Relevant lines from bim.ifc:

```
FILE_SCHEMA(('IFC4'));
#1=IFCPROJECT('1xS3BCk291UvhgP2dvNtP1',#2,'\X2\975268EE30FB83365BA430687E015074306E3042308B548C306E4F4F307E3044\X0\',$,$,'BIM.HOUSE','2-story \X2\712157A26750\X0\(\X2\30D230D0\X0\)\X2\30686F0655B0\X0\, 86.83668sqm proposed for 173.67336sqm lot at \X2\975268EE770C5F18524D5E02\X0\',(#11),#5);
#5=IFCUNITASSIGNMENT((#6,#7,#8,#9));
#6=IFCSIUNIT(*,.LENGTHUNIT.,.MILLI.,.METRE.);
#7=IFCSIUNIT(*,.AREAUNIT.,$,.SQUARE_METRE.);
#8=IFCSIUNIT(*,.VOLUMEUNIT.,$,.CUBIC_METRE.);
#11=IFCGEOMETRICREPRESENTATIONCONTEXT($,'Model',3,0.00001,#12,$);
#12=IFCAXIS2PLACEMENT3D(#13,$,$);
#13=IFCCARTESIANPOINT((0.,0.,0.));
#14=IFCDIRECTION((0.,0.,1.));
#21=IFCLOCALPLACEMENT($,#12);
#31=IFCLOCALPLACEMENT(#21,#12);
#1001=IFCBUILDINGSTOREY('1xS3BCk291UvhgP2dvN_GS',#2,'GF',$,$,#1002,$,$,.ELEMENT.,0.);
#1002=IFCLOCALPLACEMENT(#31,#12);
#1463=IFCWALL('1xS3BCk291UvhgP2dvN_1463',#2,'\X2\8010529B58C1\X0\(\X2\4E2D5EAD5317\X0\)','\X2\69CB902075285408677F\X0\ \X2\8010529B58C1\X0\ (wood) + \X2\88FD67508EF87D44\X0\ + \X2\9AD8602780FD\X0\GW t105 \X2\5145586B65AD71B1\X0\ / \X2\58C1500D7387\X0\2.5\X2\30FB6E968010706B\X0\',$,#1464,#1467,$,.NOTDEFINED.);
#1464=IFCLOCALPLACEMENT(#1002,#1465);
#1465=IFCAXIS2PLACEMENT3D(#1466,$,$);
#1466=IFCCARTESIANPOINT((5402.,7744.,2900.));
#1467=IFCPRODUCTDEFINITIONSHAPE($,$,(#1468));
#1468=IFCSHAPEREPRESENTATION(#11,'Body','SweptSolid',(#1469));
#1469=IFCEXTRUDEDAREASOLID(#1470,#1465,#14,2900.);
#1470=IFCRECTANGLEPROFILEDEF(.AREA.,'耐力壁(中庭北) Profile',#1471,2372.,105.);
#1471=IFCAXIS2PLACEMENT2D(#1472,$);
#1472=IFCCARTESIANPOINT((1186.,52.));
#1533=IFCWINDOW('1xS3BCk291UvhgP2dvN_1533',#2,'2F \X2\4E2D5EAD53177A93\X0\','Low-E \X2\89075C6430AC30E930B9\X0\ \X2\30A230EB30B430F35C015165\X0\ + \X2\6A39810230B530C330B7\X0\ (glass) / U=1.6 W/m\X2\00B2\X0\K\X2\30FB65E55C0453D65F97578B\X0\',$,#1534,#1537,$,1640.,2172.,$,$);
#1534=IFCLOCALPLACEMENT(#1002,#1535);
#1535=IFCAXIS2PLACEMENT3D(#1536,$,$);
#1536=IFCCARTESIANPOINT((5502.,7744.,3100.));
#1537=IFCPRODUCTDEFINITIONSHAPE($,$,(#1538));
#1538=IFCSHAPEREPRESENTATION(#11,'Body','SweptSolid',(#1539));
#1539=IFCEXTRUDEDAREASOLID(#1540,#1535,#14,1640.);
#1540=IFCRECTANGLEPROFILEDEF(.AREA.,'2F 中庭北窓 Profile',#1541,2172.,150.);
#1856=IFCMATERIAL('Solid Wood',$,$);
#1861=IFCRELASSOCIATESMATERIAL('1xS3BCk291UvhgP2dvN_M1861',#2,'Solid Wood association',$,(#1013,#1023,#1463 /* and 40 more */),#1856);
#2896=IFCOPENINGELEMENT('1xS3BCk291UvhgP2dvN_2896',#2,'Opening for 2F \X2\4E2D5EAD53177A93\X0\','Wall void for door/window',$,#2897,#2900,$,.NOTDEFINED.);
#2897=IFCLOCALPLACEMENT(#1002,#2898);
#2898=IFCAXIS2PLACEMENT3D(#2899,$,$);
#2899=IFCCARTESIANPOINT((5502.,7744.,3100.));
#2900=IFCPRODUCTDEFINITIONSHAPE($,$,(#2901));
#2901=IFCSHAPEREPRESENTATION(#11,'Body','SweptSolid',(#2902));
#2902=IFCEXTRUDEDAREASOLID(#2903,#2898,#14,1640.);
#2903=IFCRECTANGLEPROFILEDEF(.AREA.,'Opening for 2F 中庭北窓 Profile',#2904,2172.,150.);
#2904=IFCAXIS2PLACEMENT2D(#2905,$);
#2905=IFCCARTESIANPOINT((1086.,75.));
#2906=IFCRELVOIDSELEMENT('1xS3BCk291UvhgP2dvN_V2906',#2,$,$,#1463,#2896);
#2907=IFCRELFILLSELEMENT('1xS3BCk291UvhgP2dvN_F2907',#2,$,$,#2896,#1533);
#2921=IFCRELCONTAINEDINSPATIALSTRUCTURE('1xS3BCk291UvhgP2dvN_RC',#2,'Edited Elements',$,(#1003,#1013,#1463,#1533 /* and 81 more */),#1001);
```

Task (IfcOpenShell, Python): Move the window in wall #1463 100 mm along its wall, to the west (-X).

```python
import ifcopenshell
import ifcopenshell.api.geometry
import ifcopenshell.util.placement
import ifcopenshell.util.unit

model = ifcopenshell.open("bim.ifc")
unit_scale = ifcopenshell.util.unit.calculate_unit_scale(model)

window = model.by_guid("1xS3BCk291UvhgP2dvN_1533")
opening = window.FillsVoids[0].RelatingOpeningElement
wall = opening.VoidsElements[0].RelatingBuildingElement

wall_matrix = ifcopenshell.util.placement.get_local_placement(wall.ObjectPlacement)
shift = wall_matrix[:3, 0] * -0.1 / unit_scale
before = ifcopenshell.util.placement.get_local_placement(window.ObjectPlacement)[:3, 3].copy()

# The window is not placed relative to its opening, so move both.
for product in (opening, window):
    matrix = ifcopenshell.util.placement.get_local_placement(product.ObjectPlacement)
    matrix[:3, 3] += shift
    ifcopenshell.api.geometry.edit_object_placement(model, product=product, matrix=matrix, is_si=False)

after = ifcopenshell.util.placement.get_local_placement(window.ObjectPlacement)[:3, 3]
print("window moved by", (after - before).round(3) + 0.0)

model.write("bim_v2.ifc")
```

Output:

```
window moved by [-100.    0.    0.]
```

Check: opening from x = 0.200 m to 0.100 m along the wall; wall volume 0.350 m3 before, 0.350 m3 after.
